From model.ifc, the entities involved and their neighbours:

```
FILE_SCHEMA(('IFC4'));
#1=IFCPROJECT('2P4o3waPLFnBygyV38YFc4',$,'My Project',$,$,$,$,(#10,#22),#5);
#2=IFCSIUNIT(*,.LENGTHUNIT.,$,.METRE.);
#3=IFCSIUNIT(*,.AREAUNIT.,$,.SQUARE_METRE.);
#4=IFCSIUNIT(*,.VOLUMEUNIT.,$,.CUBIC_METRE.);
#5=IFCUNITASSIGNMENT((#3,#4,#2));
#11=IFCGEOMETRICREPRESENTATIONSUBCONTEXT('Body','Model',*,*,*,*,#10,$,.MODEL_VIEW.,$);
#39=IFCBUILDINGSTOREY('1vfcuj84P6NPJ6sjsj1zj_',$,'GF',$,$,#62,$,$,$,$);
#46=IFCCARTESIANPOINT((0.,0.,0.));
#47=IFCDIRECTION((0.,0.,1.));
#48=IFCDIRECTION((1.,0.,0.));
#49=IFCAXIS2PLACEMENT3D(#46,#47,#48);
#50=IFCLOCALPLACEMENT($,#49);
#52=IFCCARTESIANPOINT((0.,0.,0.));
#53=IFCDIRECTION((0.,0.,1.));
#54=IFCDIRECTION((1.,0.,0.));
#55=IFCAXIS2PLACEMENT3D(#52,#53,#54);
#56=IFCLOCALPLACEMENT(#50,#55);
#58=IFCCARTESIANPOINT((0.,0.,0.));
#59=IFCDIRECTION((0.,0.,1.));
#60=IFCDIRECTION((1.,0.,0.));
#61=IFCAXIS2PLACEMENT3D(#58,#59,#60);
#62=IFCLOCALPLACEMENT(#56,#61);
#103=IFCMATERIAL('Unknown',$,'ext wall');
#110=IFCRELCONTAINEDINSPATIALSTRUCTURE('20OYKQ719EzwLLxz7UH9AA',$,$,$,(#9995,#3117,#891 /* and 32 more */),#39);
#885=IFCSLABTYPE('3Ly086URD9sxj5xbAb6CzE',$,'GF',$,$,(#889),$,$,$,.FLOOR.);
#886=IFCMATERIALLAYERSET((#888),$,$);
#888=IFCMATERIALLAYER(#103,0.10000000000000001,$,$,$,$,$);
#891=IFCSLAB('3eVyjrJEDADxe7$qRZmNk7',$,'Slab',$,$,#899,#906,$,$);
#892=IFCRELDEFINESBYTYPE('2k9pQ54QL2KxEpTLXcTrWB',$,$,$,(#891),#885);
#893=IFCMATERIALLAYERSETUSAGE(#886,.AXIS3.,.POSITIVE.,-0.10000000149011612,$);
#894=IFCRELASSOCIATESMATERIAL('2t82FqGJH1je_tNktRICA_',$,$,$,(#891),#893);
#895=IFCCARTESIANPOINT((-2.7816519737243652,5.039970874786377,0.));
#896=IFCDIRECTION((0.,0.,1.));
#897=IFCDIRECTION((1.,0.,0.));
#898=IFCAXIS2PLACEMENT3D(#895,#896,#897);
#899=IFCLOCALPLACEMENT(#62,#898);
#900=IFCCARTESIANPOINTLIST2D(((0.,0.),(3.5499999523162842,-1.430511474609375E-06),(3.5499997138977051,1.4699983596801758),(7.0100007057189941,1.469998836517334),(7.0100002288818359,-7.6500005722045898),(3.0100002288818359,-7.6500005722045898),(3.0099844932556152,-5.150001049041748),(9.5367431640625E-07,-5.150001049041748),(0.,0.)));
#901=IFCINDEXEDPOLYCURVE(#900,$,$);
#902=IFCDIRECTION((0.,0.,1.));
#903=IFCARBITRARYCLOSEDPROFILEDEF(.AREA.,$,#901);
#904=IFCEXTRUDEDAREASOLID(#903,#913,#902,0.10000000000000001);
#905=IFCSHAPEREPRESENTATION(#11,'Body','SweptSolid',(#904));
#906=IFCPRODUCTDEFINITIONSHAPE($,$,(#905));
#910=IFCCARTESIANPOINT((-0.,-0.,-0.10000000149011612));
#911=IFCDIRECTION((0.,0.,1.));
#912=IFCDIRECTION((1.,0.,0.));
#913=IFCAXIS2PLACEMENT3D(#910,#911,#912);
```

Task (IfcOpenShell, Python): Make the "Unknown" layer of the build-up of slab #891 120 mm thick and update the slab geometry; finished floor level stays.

```python
import ifcopenshell
import ifcopenshell.util.element
import ifcopenshell.util.representation
import ifcopenshell.util.unit

model = ifcopenshell.open("model.ifc")
unit_scale = ifcopenshell.util.unit.calculate_unit_scale(model)

layer_set = model.by_id(886)
layer = next(l for l in layer_set.MaterialLayers if l.Material and l.Material.Name == "Unknown")
change = 0.12 / unit_scale - layer.LayerThickness
layer.LayerThickness += change

# Geometry does not follow the layer set by itself.
slabs = [e for e in ifcopenshell.util.element.get_elements_by_material(model, layer_set) if e.is_a("IfcSlab")]
for slab in sorted(slabs, key=lambda e: e.id()):
    body = ifcopenshell.util.representation.get_representation(slab, "Model", "Body")
    solid = body.Items[0]
    old_depth = solid.Depth
    solid.Depth += change
    # Extruded upwards: lower the start of the extrusion so the top stays.
    x, y, z = solid.Position.Location.Coordinates
    solid.Position.Location = model.createIfcCartesianPoint((x, y, z - change))
    print(slab.id(), f"{old_depth:g} -> {solid.Depth:g}")

# The layers are counted up from the underside, which has moved.
for usage in {ifcopenshell.util.element.get_material(slab) for slab in slabs}:
    usage.OffsetFromReferenceLine -= change

model.write("model_v2.ifc")
```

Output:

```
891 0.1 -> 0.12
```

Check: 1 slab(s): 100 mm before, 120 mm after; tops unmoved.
